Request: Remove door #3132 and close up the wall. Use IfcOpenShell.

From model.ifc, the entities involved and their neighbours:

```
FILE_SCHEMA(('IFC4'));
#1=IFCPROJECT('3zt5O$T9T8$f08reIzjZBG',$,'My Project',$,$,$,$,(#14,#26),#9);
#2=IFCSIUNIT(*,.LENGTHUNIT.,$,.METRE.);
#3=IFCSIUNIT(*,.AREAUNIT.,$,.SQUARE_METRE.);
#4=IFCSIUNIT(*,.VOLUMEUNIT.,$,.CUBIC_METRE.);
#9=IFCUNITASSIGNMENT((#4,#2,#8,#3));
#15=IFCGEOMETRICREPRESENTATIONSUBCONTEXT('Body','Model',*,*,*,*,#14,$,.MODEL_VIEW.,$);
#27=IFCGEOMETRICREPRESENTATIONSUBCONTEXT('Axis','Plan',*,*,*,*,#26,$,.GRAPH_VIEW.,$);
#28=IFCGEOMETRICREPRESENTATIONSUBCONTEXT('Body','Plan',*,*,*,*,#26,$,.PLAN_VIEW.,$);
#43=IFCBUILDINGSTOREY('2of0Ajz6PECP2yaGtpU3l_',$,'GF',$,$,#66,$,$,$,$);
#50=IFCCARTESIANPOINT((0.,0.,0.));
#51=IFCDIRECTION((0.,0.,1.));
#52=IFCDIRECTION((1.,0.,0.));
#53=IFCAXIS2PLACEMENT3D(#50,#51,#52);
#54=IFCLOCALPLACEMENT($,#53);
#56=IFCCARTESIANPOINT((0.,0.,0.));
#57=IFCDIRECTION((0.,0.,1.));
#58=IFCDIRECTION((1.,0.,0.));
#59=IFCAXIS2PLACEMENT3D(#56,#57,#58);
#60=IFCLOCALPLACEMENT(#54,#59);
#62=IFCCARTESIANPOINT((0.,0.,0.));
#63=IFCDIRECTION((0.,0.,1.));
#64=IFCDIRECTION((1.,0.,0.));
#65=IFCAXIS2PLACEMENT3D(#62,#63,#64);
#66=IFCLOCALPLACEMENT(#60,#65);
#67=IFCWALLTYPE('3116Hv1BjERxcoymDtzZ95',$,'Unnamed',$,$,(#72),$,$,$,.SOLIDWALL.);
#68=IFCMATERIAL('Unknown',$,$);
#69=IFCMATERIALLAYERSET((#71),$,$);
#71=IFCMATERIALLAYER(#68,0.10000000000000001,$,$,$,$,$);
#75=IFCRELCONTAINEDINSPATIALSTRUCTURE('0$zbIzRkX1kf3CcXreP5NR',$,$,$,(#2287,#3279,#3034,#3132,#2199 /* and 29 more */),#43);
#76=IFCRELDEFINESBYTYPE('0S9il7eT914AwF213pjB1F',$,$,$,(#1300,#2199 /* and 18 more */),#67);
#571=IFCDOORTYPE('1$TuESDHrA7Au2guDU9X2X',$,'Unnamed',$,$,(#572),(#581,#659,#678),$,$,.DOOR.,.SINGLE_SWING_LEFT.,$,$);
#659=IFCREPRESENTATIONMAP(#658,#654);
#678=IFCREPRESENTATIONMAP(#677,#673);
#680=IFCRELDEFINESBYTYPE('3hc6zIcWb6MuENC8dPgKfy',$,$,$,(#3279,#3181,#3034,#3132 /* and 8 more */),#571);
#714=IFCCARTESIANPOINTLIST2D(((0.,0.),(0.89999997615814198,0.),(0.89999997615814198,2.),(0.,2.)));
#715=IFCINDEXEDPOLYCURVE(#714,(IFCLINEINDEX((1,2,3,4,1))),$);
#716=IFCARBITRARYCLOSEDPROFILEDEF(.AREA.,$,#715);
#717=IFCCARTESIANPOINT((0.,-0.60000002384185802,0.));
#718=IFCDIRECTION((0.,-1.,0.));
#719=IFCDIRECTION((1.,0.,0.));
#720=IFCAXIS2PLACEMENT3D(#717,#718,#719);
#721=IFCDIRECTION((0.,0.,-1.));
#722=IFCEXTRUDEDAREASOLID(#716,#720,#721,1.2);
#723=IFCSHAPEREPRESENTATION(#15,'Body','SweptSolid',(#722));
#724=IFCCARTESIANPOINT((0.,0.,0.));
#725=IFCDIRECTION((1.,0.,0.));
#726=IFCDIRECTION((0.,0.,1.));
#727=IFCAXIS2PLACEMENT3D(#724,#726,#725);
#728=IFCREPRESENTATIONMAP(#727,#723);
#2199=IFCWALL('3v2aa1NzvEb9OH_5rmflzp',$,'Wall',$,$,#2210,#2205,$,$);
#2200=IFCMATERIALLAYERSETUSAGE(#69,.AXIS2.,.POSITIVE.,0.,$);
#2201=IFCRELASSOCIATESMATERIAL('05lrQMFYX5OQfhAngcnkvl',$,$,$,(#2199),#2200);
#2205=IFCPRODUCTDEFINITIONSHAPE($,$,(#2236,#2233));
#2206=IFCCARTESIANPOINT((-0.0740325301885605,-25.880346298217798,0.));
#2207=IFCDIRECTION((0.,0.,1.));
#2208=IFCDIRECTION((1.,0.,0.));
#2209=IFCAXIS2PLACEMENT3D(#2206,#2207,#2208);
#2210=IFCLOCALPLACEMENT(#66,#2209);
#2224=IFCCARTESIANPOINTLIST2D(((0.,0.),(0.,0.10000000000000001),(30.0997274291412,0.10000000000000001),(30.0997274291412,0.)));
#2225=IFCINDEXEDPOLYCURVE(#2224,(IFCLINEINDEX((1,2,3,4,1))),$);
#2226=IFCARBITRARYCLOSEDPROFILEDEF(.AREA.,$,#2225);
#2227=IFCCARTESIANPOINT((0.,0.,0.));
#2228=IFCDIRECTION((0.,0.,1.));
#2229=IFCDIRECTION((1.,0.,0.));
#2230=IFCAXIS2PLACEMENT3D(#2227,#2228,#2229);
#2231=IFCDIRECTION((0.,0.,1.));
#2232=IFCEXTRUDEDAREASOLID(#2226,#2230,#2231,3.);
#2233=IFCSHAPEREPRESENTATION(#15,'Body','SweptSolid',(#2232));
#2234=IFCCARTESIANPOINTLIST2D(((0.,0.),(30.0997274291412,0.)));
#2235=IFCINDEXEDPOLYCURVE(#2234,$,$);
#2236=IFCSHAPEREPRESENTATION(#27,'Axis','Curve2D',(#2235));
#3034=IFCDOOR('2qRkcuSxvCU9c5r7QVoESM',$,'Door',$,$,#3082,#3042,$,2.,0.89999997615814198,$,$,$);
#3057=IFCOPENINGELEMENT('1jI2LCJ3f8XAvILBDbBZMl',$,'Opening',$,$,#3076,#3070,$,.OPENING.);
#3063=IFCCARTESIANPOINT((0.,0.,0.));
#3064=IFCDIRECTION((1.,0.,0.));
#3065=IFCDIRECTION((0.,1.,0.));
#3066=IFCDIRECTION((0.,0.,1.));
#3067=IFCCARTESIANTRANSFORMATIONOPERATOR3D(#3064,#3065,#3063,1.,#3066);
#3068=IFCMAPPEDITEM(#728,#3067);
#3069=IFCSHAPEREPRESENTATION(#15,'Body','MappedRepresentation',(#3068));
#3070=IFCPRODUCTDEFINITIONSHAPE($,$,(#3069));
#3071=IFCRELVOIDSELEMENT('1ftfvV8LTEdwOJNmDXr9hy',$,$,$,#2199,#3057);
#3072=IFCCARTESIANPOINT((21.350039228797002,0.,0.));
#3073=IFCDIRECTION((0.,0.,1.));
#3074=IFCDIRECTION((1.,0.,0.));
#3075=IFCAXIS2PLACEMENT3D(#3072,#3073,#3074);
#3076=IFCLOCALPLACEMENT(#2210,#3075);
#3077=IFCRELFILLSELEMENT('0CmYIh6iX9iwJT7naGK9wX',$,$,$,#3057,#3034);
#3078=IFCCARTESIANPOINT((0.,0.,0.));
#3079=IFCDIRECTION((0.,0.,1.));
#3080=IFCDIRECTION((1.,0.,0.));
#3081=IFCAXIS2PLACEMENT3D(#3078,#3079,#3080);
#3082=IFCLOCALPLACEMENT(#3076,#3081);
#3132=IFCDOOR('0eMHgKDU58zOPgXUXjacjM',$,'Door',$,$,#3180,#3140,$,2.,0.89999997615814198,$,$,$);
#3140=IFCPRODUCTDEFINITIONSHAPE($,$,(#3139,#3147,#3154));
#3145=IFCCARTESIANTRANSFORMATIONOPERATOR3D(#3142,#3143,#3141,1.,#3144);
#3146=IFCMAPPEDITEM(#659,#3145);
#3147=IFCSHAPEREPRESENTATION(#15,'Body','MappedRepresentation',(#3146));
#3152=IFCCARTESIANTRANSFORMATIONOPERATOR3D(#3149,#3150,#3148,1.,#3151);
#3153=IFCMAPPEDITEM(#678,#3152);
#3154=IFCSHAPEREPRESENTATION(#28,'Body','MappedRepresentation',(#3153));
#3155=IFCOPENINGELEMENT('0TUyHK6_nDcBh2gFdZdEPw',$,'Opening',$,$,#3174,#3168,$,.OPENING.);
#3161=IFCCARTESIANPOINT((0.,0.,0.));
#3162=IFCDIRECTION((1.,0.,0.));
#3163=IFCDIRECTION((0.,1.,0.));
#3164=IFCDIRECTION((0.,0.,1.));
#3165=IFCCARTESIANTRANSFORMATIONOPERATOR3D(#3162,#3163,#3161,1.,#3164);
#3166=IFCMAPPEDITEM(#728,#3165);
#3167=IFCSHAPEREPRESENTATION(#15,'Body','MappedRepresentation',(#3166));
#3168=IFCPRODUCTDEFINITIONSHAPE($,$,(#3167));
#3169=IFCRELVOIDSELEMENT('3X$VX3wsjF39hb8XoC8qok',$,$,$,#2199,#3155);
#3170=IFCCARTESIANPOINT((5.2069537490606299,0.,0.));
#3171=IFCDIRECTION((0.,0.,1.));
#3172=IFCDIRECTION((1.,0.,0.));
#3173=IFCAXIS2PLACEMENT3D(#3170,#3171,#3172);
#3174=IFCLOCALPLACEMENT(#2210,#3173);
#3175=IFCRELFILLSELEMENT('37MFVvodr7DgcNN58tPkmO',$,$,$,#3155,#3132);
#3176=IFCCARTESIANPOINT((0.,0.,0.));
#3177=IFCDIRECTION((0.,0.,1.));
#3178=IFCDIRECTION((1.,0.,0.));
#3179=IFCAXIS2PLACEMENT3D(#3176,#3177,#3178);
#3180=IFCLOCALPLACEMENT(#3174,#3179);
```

```python
import ifcopenshell
import ifcopenshell.api.feature
import ifcopenshell.api.root
import ifcopenshell.geom
import ifcopenshell.util.shape

model = ifcopenshell.open("model.ifc")
settings = ifcopenshell.geom.settings()


def volume(element):
    """Net volume in cubic metres, openings subtracted."""
    shape = ifcopenshell.geom.create_shape(settings, element)
    return ifcopenshell.util.shape.get_volume(shape.geometry)


door = model.by_guid("0eMHgKDU58zOPgXUXjacjM")
opening = door.FillsVoids[0].RelatingOpeningElement
wall = opening.VoidsElements[0].RelatingBuildingElement
before = volume(wall)

ifcopenshell.api.root.remove_product(model, product=door)
ifcopenshell.api.feature.remove_feature(model, feature=opening)

after = volume(wall)

print(f"wall volume {before:.3f} -> {after:.3f} m3")

model.write("model_v2.ifc")
```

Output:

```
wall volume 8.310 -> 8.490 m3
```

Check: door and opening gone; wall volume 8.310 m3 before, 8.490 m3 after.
